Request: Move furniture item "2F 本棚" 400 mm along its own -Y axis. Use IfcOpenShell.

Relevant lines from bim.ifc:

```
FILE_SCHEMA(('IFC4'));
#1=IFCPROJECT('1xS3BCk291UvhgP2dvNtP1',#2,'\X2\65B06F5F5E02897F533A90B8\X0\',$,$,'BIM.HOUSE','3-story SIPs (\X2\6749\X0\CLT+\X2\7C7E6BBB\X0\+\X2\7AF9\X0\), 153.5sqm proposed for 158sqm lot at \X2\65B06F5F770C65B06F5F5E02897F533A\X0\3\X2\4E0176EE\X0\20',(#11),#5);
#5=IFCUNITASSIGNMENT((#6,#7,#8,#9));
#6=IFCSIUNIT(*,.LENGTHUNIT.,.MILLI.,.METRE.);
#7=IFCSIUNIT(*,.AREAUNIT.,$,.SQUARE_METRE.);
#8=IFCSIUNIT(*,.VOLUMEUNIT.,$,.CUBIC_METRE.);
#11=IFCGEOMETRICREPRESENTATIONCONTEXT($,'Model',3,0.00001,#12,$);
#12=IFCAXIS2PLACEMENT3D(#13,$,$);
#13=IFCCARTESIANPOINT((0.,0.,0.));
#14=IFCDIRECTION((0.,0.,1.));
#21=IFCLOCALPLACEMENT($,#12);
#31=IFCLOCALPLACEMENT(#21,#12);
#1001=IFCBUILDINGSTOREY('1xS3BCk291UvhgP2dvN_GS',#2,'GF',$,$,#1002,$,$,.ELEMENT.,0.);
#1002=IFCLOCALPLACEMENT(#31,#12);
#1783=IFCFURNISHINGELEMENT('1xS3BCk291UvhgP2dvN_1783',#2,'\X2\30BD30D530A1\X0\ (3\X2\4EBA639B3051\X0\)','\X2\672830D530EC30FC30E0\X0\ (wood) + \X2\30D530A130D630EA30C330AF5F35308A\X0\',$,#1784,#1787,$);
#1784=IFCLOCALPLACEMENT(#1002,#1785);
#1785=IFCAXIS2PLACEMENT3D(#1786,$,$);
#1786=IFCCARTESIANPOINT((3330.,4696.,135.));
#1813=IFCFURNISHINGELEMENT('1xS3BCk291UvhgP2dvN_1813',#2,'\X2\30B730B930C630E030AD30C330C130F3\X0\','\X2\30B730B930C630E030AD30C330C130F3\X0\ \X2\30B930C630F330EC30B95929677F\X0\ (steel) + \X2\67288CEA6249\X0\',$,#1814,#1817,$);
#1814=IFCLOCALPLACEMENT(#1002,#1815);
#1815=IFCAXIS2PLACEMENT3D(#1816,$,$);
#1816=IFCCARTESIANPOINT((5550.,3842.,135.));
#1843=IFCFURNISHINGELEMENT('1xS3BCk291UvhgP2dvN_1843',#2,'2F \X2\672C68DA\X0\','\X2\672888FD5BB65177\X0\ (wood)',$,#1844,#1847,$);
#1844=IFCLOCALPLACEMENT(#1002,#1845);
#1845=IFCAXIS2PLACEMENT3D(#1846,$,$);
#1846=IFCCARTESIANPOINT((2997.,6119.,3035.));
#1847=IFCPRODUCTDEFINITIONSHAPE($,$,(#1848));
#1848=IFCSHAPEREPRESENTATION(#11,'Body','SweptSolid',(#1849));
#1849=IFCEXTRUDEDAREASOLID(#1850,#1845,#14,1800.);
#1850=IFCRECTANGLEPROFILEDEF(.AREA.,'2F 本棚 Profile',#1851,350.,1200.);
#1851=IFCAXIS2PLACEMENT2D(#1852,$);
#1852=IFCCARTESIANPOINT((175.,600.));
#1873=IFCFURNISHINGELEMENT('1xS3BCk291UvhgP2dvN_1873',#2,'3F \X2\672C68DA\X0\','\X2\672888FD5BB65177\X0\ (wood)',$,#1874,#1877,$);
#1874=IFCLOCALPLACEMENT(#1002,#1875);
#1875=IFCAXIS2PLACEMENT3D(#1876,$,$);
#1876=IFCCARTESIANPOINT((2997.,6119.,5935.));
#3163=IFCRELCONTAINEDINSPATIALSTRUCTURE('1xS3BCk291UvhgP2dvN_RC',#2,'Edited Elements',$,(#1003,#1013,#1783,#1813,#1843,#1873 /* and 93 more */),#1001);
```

```python
import ifcopenshell
import ifcopenshell.api.geometry
import ifcopenshell.util.placement
import ifcopenshell.util.unit

model = ifcopenshell.open("bim.ifc")
unit_scale = ifcopenshell.util.unit.calculate_unit_scale(model)

item = model.by_guid("1xS3BCk291UvhgP2dvN_1843")
matrix = ifcopenshell.util.placement.get_local_placement(item.ObjectPlacement)
matrix[:3, 3] -= matrix[:3, 1] * 0.4 / unit_scale
ifcopenshell.api.geometry.edit_object_placement(model, product=item, matrix=matrix, is_si=False)

print(ifcopenshell.util.placement.get_local_placement(item.ObjectPlacement).round(3) + 0.0)

model.write("bim_edited.ifc")
```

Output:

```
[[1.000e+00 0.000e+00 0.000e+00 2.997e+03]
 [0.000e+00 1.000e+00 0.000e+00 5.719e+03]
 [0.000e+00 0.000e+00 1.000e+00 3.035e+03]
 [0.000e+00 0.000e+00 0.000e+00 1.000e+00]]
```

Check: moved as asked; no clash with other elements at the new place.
